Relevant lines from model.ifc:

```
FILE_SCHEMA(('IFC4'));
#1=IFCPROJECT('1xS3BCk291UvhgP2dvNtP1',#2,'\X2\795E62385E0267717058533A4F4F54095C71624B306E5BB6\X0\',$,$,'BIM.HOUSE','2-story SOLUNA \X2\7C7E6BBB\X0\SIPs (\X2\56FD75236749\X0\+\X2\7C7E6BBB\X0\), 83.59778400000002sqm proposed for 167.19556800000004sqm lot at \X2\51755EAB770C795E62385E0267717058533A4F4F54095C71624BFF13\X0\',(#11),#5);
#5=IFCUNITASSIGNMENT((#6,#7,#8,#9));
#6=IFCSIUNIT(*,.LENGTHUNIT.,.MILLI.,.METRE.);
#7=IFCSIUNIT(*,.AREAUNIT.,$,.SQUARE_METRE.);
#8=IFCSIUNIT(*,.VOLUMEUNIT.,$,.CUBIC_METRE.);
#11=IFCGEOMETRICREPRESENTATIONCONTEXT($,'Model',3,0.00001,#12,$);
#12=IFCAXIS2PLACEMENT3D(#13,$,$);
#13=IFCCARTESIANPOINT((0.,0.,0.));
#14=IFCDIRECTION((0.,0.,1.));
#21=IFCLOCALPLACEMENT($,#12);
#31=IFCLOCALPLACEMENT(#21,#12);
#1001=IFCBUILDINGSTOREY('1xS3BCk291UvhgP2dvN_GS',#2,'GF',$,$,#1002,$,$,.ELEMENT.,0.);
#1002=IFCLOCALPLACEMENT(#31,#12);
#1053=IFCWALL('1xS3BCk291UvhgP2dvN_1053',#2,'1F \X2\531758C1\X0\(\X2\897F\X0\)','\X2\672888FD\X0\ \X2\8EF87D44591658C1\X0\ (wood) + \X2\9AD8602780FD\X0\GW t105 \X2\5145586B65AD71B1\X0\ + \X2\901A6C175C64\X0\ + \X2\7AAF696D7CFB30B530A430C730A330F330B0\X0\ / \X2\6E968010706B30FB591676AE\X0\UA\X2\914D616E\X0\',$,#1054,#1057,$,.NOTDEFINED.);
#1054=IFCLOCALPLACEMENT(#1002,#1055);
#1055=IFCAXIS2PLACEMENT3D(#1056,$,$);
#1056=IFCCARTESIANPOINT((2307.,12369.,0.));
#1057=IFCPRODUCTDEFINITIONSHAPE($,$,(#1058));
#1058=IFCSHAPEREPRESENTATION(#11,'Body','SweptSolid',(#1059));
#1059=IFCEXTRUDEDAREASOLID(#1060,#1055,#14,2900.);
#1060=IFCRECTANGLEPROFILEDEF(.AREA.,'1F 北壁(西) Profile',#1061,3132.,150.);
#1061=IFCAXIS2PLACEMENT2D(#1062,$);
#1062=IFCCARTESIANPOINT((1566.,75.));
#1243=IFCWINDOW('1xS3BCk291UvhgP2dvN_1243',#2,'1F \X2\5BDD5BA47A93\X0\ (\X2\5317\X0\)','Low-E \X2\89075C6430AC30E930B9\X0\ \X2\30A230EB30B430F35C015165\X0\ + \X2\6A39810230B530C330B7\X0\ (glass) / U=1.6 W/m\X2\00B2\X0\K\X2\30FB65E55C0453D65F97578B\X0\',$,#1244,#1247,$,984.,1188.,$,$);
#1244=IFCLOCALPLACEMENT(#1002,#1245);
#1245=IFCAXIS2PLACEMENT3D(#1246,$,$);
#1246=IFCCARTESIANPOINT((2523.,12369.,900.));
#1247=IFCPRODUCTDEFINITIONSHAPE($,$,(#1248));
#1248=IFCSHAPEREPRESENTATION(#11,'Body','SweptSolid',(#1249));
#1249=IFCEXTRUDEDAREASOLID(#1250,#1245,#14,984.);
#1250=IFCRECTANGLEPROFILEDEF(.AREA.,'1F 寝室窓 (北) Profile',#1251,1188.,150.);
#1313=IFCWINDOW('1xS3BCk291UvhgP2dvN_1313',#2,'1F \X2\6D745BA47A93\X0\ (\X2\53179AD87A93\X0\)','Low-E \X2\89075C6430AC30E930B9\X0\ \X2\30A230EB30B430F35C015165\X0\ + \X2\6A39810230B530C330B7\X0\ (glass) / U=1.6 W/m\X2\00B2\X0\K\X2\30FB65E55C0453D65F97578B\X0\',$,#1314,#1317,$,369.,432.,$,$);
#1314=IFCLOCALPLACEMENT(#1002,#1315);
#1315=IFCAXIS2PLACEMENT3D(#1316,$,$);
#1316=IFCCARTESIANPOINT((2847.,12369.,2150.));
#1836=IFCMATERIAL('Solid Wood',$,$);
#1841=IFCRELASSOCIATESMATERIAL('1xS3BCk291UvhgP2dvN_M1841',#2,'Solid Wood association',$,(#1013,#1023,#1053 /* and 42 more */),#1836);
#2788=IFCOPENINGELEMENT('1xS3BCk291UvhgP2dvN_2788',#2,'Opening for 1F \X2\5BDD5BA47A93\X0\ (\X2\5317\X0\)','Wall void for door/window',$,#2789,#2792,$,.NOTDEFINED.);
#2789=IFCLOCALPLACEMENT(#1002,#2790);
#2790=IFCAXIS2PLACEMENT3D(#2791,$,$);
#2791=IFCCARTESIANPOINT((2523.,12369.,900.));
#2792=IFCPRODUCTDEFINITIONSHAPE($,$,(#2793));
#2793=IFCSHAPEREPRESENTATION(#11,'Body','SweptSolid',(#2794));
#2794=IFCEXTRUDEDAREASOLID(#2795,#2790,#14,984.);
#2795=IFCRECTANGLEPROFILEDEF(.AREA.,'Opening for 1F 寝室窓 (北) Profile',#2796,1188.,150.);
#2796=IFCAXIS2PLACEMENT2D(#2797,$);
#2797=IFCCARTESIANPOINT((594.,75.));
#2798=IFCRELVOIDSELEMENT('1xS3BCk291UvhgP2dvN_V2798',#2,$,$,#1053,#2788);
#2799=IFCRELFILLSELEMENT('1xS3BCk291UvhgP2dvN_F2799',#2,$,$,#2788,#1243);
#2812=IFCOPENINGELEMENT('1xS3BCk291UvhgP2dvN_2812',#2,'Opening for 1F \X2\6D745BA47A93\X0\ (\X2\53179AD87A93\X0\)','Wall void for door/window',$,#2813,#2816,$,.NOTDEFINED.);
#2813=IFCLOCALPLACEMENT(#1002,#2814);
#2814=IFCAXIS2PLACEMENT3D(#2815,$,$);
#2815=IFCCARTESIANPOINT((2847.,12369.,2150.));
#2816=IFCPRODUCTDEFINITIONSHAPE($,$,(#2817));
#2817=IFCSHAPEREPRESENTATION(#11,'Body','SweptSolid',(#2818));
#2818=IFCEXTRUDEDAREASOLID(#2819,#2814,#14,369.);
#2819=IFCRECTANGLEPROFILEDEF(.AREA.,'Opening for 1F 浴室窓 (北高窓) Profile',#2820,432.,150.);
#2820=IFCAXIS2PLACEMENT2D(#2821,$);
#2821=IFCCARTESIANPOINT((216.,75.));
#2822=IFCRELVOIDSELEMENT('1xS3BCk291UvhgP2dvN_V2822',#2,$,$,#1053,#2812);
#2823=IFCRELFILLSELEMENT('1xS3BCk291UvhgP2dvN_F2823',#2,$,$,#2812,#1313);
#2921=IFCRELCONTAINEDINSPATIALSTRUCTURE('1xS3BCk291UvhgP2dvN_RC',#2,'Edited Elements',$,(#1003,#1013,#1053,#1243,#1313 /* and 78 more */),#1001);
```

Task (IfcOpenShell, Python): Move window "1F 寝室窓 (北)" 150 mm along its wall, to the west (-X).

```python
import ifcopenshell
import ifcopenshell.api.geometry
import ifcopenshell.util.placement
import ifcopenshell.util.unit

model = ifcopenshell.open("model.ifc")
unit_scale = ifcopenshell.util.unit.calculate_unit_scale(model)

window = model.by_guid("1xS3BCk291UvhgP2dvN_1243")
opening = window.FillsVoids[0].RelatingOpeningElement
wall = opening.VoidsElements[0].RelatingBuildingElement

wall_matrix = ifcopenshell.util.placement.get_local_placement(wall.ObjectPlacement)
shift = wall_matrix[:3, 0] * -0.15 / unit_scale
before = ifcopenshell.util.placement.get_local_placement(window.ObjectPlacement)[:3, 3].copy()

# The window is not placed relative to its opening, so move both.
for product in (opening, window):
    matrix = ifcopenshell.util.placement.get_local_placement(product.ObjectPlacement)
    matrix[:3, 3] += shift
    ifcopenshell.api.geometry.edit_object_placement(model, product=product, matrix=matrix, is_si=False)

after = ifcopenshell.util.placement.get_local_placement(window.ObjectPlacement)[:3, 3]
print("window moved by", (after - before).round(3) + 0.0)

model.write("model-out.ifc")
```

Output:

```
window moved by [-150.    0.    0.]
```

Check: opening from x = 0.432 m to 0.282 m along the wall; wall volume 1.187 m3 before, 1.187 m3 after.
